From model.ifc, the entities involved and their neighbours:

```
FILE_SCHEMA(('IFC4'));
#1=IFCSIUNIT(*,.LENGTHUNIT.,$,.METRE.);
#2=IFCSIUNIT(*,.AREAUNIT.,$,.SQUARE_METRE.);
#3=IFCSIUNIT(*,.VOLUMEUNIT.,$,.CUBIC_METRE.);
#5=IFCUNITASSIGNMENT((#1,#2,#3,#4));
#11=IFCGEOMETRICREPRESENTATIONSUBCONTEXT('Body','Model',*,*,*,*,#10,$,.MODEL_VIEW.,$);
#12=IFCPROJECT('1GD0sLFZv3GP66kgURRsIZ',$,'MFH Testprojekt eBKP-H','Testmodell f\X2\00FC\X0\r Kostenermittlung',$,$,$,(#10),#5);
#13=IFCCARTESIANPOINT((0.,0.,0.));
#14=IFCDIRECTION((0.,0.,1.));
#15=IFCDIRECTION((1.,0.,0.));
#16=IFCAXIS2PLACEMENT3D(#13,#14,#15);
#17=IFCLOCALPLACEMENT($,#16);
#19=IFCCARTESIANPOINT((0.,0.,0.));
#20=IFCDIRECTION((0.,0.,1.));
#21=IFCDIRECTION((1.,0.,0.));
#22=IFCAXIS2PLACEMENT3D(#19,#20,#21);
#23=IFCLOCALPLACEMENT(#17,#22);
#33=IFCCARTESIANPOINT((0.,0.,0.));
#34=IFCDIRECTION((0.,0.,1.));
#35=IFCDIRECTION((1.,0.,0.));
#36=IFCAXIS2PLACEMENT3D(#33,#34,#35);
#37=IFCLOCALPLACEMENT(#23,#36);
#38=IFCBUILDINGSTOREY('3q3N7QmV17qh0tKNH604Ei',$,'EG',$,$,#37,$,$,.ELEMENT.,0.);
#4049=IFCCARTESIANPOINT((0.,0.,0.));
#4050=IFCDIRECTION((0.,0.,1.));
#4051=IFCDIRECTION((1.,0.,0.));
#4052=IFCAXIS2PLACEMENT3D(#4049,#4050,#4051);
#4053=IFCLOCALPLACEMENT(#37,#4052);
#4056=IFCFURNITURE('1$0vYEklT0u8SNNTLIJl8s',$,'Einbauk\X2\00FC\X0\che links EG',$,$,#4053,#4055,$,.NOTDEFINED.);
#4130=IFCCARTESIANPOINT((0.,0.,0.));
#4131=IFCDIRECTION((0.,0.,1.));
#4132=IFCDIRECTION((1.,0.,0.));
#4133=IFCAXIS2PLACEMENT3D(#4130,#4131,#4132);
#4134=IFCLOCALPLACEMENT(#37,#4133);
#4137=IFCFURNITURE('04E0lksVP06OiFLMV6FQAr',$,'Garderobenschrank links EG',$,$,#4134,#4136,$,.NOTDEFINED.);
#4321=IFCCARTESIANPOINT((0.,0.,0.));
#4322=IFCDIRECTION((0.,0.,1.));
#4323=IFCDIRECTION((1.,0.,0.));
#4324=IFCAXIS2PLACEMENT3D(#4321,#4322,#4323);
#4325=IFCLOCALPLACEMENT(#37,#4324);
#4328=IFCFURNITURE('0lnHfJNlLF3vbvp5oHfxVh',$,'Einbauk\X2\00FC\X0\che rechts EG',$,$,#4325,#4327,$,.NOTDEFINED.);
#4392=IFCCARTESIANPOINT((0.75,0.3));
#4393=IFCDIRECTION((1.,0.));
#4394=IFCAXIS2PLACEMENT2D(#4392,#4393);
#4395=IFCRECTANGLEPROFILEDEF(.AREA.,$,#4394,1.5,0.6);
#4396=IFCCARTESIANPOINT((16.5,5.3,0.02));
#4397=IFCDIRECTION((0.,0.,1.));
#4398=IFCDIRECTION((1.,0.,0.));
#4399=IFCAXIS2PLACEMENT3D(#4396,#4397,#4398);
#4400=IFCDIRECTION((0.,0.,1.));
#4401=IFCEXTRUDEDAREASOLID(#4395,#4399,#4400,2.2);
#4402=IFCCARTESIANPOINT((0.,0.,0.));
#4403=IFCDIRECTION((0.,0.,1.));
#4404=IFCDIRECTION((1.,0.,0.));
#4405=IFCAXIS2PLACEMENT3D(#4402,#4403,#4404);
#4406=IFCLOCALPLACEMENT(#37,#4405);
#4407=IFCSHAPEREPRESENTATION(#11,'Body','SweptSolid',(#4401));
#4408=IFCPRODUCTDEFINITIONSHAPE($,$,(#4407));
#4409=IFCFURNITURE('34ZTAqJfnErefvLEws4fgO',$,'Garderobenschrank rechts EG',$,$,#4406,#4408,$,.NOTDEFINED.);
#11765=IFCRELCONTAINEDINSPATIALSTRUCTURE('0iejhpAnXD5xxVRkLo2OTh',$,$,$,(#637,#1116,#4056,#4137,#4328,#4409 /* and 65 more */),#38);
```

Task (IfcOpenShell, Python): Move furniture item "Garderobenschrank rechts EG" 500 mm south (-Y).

```python
import ifcopenshell
import ifcopenshell.api.geometry
import ifcopenshell.util.placement
import ifcopenshell.util.unit

model = ifcopenshell.open("model.ifc")
unit_scale = ifcopenshell.util.unit.calculate_unit_scale(model)

item = model.by_guid("34ZTAqJfnErefvLEws4fgO")
matrix = ifcopenshell.util.placement.get_local_placement(item.ObjectPlacement)
matrix[1, 3] -= 0.5 / unit_scale
ifcopenshell.api.geometry.edit_object_placement(model, product=item, matrix=matrix, is_si=False)

print(ifcopenshell.util.placement.get_local_placement(item.ObjectPlacement).round(3) + 0.0)

model.write("model_updated.ifc")
```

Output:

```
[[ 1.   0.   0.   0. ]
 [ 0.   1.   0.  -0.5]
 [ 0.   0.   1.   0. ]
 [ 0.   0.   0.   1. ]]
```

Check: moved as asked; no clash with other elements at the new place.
